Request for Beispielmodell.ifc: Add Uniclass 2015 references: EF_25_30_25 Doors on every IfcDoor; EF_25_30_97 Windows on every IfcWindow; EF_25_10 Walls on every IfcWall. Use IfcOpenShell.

First a look at what the model holds.

```python
import ifcopenshell

model = ifcopenshell.open("Beispielmodell.ifc")
print(model.schema)
print("classifications:", [c.Name for c in model.by_type("IfcClassification")])
for ifc_class in ("IfcDoor", "IfcRoof", "IfcStair", "IfcWall", "IfcWindow"):
    print(ifc_class, len(model.by_type(ifc_class)))
```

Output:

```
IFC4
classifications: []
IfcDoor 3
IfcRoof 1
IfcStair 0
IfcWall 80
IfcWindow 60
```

```python
import ifcopenshell
import ifcopenshell.api.classification

model = ifcopenshell.open("Beispielmodell.ifc")

system = ifcopenshell.api.classification.add_classification(model, classification="Uniclass 2015")

codes = {
    "IfcDoor": ("EF_25_30_25", "Doors"),
    "IfcWindow": ("EF_25_30_97", "Windows"),
    "IfcWall": ("EF_25_10", "Walls"),
}
for ifc_class, (code, name) in codes.items():
    products = model.by_type(ifc_class)
    ifcopenshell.api.classification.add_reference(
        model, products=products, classification=system, identification=code, name=name
    )
    print(code, len(products))

model.write("Beispielmodell_v2.ifc")
```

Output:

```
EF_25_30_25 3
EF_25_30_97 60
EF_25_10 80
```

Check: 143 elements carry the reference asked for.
